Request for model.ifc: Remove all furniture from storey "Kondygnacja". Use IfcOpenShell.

First a look at what the model holds.

```python
import ifcopenshell
import ifcopenshell.util.element

model = ifcopenshell.open("model.ifc")
print(model.schema)
storey = next(s for s in model.by_type("IfcBuildingStorey") if s.Name == "Kondygnacja")
furniture = [e for e in ifcopenshell.util.element.get_decomposition(storey) if e.is_a("IfcFurnishingElement")]
seen = {}
for e in furniture:
    element_type = ifcopenshell.util.element.get_type(e)
    name = element_type.Name if element_type not in (None, e) else None
    seen[name] = seen.get(name, 0) + 1
for name, count in sorted(seen.items(), key=str):
    print(count, "x", name)
```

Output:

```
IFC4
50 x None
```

```python
import ifcopenshell
import ifcopenshell.api.root
import ifcopenshell.util.element

model = ifcopenshell.open("model.ifc")

storey = next(s for s in model.by_type("IfcBuildingStorey") if s.Name == "Kondygnacja")
furniture = [e for e in ifcopenshell.util.element.get_decomposition(storey) if e.is_a("IfcFurnishingElement")]

for e in furniture:
    ifcopenshell.api.root.remove_product(model, product=e)
print(len(furniture), "removed")

model.write("model_v2.ifc")
```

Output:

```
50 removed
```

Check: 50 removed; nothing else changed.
